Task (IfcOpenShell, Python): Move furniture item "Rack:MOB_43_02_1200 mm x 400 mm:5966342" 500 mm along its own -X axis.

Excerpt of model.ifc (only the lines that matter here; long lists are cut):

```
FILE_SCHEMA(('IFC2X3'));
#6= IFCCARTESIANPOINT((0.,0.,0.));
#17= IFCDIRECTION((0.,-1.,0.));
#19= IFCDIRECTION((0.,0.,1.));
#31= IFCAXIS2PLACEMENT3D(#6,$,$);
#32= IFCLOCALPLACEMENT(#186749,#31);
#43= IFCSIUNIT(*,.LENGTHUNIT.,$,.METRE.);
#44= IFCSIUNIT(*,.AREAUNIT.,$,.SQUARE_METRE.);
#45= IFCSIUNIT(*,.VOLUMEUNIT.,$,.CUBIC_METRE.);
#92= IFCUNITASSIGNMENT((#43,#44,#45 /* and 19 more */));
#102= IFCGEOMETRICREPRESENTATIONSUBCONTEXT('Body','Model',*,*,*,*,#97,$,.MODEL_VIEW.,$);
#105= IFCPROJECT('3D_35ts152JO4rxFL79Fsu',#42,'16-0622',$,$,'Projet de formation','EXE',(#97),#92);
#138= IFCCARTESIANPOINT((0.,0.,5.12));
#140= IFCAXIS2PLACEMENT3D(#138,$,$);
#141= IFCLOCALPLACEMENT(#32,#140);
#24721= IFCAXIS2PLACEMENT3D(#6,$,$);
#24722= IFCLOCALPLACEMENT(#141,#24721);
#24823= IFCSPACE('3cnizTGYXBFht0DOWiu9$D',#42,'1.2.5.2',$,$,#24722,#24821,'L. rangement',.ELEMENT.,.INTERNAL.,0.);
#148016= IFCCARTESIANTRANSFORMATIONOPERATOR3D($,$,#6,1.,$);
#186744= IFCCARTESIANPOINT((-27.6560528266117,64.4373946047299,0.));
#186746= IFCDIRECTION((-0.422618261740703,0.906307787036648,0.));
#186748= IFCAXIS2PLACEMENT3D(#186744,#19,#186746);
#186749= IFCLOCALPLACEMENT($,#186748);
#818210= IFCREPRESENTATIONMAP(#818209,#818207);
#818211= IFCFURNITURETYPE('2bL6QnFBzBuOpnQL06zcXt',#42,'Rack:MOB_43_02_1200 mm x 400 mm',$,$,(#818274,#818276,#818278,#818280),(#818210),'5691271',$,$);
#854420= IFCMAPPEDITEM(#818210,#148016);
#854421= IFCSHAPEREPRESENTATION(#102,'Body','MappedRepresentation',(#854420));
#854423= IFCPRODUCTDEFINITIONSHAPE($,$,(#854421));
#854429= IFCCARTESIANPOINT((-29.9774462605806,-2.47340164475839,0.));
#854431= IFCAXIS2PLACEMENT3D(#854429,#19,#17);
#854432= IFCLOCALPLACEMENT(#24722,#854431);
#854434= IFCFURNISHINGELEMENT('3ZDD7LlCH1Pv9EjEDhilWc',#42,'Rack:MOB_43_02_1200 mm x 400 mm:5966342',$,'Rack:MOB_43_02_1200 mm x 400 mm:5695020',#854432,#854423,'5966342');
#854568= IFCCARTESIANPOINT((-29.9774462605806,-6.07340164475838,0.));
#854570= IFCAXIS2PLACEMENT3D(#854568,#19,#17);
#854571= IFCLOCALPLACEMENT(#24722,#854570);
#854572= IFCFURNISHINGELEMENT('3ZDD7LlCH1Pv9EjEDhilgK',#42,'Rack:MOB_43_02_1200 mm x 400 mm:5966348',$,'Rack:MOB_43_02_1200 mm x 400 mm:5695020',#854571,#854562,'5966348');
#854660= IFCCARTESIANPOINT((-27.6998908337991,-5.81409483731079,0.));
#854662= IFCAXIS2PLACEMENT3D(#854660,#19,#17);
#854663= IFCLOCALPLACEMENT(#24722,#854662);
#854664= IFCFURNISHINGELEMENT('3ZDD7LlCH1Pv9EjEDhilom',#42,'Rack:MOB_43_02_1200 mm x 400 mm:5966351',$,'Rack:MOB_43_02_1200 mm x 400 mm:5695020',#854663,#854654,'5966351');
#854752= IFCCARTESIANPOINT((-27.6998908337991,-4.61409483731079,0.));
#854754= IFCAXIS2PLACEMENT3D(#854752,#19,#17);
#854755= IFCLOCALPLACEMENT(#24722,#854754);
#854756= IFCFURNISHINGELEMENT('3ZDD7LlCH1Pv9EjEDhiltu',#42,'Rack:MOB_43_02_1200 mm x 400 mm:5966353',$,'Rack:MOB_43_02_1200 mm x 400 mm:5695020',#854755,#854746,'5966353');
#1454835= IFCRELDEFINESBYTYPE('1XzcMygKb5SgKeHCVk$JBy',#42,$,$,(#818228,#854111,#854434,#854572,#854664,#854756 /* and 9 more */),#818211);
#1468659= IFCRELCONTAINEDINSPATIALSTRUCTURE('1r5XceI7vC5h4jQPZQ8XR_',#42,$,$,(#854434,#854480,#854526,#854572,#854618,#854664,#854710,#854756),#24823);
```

```python
import ifcopenshell
import ifcopenshell.api.geometry
import ifcopenshell.util.placement
import ifcopenshell.util.unit

model = ifcopenshell.open("model.ifc")
unit_scale = ifcopenshell.util.unit.calculate_unit_scale(model)

item = model.by_guid("3ZDD7LlCH1Pv9EjEDhilWc")
matrix = ifcopenshell.util.placement.get_local_placement(item.ObjectPlacement)
matrix[:3, 3] -= matrix[:3, 0] * 0.5 / unit_scale
ifcopenshell.api.geometry.edit_object_placement(model, product=item, matrix=matrix, is_si=False)

print(ifcopenshell.util.placement.get_local_placement(item.ObjectPlacement).round(3) + 0.0)

model.write("model-out.ifc")
```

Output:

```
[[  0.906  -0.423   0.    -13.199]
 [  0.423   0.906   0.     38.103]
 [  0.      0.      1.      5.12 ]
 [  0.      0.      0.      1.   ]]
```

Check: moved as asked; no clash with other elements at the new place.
